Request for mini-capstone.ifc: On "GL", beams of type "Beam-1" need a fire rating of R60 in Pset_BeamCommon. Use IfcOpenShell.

First a look at what the model holds.

```python
import ifcopenshell
import ifcopenshell.util.element

model = ifcopenshell.open("mini-capstone.ifc")
print(model.schema)
storey = next(s for s in model.by_type("IfcBuildingStorey") if s.Name == "GL")
beams = [e for e in ifcopenshell.util.element.get_decomposition(storey) if e.is_a("IfcBeam")]
seen = {}
for e in beams:
    element_type = ifcopenshell.util.element.get_type(e)
    key = (element_type.Name if element_type != e and element_type else None, ifcopenshell.util.element.get_pset(e, "Pset_BeamCommon", "FireRating"))
    seen[key] = seen.get(key, 0) + 1
for (name, value), count in sorted(seen.items(), key=str):
    print(count, "x", name, "|", value)
```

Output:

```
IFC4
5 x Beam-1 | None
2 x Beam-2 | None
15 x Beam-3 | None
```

```python
import ifcopenshell
import ifcopenshell.api.pset
import ifcopenshell.util.element

model = ifcopenshell.open("mini-capstone.ifc")

storey = next(s for s in model.by_type("IfcBuildingStorey") if s.Name == "GL")
beams = [e for e in ifcopenshell.util.element.get_decomposition(storey) if e.is_a("IfcBeam")]

count = 0
for e in beams:
    element_type = ifcopenshell.util.element.get_type(e)
    if element_type in (None, e) or element_type.Name != "Beam-1":
        continue
    # add_pset returns the element's existing set when there is one.
    pset = ifcopenshell.api.pset.add_pset(model, product=e, name="Pset_BeamCommon")
    ifcopenshell.api.pset.edit_pset(model, pset=pset, properties={"FireRating": "R60"})
    count += 1

print(count, "beams updated")

model.write("mini-capstone-out.ifc")
```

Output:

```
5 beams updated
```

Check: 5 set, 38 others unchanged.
